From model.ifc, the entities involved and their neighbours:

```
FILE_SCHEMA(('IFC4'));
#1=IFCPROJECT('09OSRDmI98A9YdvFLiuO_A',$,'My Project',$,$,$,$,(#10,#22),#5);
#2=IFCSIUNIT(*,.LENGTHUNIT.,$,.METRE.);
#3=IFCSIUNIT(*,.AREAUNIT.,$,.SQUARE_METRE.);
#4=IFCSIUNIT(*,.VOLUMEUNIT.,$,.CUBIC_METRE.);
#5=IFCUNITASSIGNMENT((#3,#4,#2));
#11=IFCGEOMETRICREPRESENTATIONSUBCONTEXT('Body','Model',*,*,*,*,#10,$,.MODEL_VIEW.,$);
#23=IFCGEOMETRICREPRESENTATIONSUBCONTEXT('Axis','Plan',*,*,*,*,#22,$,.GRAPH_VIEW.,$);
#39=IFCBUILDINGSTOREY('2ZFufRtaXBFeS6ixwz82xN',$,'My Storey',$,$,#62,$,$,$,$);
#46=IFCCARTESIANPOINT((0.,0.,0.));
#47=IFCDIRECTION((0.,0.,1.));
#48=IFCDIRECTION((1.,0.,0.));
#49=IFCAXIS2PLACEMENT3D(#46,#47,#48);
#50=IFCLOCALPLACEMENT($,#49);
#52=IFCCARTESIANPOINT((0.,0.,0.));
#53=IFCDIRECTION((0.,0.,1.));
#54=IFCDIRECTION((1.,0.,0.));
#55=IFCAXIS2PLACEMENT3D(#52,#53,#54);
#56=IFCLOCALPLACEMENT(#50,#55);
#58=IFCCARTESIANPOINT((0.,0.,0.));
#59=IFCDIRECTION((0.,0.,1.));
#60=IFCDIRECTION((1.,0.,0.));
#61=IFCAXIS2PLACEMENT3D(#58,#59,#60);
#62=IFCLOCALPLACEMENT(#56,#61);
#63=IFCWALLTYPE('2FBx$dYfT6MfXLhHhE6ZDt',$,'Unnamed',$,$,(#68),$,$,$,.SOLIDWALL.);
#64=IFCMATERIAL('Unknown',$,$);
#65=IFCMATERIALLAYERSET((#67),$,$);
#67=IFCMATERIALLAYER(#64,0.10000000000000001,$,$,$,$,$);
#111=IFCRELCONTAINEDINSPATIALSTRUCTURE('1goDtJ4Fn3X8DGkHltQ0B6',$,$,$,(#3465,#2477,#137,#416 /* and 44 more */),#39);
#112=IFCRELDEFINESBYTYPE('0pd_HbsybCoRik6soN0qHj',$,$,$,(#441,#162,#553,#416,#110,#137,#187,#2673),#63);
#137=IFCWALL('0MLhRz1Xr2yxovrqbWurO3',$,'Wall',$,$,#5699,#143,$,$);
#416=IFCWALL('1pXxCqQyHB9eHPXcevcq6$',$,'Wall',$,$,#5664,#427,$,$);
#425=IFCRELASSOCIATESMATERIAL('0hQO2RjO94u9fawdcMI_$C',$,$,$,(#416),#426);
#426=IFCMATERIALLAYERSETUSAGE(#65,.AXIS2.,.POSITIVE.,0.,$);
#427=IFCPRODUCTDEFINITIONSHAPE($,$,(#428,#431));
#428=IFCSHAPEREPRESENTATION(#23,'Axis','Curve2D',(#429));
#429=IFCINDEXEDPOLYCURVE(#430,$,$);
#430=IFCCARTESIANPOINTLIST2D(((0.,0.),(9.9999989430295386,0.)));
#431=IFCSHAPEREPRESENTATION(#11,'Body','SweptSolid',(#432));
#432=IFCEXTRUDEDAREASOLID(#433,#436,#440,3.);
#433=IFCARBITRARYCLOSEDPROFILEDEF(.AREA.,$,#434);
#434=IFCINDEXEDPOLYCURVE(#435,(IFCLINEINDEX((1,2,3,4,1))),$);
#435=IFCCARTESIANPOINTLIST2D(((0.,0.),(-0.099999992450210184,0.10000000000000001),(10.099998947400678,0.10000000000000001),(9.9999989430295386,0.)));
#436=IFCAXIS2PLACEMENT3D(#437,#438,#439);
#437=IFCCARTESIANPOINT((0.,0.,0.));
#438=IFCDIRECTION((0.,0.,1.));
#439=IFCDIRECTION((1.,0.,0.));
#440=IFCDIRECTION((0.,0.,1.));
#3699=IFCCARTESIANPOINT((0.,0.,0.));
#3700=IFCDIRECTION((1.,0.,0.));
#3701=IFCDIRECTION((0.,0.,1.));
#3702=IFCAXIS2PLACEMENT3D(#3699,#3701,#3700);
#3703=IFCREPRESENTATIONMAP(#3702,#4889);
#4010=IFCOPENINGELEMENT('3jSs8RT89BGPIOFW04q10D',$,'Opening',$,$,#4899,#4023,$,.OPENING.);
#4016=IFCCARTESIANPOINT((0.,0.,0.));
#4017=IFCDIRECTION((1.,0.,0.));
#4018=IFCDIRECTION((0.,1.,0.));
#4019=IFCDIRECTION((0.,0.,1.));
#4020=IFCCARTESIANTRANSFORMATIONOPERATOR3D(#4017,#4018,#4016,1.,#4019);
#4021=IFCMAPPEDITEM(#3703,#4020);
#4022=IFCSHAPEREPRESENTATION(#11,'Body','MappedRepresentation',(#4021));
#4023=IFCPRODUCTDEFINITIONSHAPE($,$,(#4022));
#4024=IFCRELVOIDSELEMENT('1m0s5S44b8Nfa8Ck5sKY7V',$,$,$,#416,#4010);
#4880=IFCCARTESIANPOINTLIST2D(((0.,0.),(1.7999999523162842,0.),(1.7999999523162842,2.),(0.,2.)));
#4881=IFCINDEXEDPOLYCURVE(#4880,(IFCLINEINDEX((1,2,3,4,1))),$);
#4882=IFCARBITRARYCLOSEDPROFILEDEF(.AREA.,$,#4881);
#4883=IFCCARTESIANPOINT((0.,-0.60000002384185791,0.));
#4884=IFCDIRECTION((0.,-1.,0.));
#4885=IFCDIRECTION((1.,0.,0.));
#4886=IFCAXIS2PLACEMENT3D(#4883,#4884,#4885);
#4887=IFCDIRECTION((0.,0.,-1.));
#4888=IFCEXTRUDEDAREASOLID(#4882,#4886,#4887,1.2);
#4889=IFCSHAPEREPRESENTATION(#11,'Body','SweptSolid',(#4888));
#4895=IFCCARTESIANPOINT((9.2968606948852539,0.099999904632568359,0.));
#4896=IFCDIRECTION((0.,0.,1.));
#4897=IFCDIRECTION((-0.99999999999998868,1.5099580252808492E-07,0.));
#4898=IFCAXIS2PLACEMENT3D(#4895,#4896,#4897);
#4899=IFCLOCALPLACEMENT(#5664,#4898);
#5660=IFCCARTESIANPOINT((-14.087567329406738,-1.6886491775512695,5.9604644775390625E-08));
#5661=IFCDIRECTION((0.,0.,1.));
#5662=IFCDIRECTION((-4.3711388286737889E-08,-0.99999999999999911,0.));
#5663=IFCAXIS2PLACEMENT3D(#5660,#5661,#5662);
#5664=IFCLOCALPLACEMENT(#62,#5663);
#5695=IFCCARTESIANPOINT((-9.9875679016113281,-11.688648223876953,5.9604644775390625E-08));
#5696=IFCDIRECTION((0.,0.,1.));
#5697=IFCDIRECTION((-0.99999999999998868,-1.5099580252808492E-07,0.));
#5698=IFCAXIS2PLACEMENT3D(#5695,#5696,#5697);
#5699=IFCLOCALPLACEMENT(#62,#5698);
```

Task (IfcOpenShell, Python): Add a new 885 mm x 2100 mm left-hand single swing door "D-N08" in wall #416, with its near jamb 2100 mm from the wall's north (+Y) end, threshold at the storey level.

```python
import numpy as np
import ifcopenshell
import ifcopenshell.api.feature
import ifcopenshell.api.geometry
import ifcopenshell.api.root
import ifcopenshell.api.spatial
import ifcopenshell.geom
import ifcopenshell.util.element
import ifcopenshell.util.placement
import ifcopenshell.util.representation
import ifcopenshell.util.shape
import ifcopenshell.util.unit

model = ifcopenshell.open("model.ifc")
unit_scale = ifcopenshell.util.unit.calculate_unit_scale(model)
settings = ifcopenshell.geom.settings()


def volume(element):
    """Net volume in cubic metres, openings subtracted."""
    shape = ifcopenshell.geom.create_shape(settings, element)
    return ifcopenshell.util.shape.get_volume(shape.geometry)


wall = model.by_id(416)
storey = ifcopenshell.util.element.get_container(wall, ifc_class="IfcBuildingStorey")
context = ifcopenshell.util.representation.get_context(model, "Model", "Body", "MODEL_VIEW")
before = volume(wall)

width, height, from_end, sill = 0.885, 2.1, 2.1, 0.0  # metres

# The wall runs along its own X axis, and the end named is its -X end.
wall_shape = ifcopenshell.geom.create_shape(settings, wall)
x, y, z = ifcopenshell.util.shape.get_vertices(wall_shape.geometry).T
start = x.min() + from_end
face, thickness = float(y.min()), float(y.max() - y.min())
wall_matrix = ifcopenshell.util.placement.get_local_placement(wall.ObjectPlacement)
level = ifcopenshell.util.placement.get_local_placement(storey.ObjectPlacement)[2, 3]


def in_wall(x, y):
    """Placement at x, y metres in the wall's axes, at sill height."""
    matrix = wall_matrix.copy()
    matrix[:, 3] = wall_matrix @ np.array([x / unit_scale, y / unit_scale, 0.0, 1.0])
    matrix[2, 3] = level + sill / unit_scale
    return matrix


# Opening: a box that overshoots both wall faces by 50 mm.
opening = ifcopenshell.api.root.create_entity(model, ifc_class="IfcOpeningElement", predefined_type="OPENING")
box = ifcopenshell.api.geometry.add_wall_representation(
    model, context=context, length=width, height=height, thickness=thickness + 0.1
)
ifcopenshell.api.geometry.assign_representation(model, product=opening, representation=box)
ifcopenshell.api.geometry.edit_object_placement(model, product=opening, matrix=in_wall(start, face - 0.05), is_si=False)
ifcopenshell.api.feature.add_feature(model, feature=opening, element=wall)

door = ifcopenshell.api.root.create_entity(model, ifc_class="IfcDoor", name="D-N08", predefined_type="DOOR")
door.OverallWidth, door.OverallHeight = width / unit_scale, height / unit_scale
door.OperationType = "SINGLE_SWING_LEFT"
body = ifcopenshell.api.geometry.add_door_representation(
    model,
    context=context,
    overall_width=door.OverallWidth,
    overall_height=door.OverallHeight,
    operation_type="SINGLE_SWING_LEFT",
    lining_properties={"LiningDepth": thickness / unit_scale, "ThresholdDepth": thickness / unit_scale},
)
ifcopenshell.api.geometry.assign_representation(model, product=door, representation=body)
ifcopenshell.api.spatial.assign_container(model, products=[door], relating_structure=storey)
ifcopenshell.api.feature.add_filling(model, opening=opening, element=door)

# The lining spans the wall, so the door starts at the wall face.
ifcopenshell.api.geometry.edit_object_placement(model, product=door, matrix=in_wall(start, face), is_si=False)

after = volume(wall)

print(f"wall volume {before:.3f} -> {after:.3f} m3")

model.write("model_rev.ifc")
```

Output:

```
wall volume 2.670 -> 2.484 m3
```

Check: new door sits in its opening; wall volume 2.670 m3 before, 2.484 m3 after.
